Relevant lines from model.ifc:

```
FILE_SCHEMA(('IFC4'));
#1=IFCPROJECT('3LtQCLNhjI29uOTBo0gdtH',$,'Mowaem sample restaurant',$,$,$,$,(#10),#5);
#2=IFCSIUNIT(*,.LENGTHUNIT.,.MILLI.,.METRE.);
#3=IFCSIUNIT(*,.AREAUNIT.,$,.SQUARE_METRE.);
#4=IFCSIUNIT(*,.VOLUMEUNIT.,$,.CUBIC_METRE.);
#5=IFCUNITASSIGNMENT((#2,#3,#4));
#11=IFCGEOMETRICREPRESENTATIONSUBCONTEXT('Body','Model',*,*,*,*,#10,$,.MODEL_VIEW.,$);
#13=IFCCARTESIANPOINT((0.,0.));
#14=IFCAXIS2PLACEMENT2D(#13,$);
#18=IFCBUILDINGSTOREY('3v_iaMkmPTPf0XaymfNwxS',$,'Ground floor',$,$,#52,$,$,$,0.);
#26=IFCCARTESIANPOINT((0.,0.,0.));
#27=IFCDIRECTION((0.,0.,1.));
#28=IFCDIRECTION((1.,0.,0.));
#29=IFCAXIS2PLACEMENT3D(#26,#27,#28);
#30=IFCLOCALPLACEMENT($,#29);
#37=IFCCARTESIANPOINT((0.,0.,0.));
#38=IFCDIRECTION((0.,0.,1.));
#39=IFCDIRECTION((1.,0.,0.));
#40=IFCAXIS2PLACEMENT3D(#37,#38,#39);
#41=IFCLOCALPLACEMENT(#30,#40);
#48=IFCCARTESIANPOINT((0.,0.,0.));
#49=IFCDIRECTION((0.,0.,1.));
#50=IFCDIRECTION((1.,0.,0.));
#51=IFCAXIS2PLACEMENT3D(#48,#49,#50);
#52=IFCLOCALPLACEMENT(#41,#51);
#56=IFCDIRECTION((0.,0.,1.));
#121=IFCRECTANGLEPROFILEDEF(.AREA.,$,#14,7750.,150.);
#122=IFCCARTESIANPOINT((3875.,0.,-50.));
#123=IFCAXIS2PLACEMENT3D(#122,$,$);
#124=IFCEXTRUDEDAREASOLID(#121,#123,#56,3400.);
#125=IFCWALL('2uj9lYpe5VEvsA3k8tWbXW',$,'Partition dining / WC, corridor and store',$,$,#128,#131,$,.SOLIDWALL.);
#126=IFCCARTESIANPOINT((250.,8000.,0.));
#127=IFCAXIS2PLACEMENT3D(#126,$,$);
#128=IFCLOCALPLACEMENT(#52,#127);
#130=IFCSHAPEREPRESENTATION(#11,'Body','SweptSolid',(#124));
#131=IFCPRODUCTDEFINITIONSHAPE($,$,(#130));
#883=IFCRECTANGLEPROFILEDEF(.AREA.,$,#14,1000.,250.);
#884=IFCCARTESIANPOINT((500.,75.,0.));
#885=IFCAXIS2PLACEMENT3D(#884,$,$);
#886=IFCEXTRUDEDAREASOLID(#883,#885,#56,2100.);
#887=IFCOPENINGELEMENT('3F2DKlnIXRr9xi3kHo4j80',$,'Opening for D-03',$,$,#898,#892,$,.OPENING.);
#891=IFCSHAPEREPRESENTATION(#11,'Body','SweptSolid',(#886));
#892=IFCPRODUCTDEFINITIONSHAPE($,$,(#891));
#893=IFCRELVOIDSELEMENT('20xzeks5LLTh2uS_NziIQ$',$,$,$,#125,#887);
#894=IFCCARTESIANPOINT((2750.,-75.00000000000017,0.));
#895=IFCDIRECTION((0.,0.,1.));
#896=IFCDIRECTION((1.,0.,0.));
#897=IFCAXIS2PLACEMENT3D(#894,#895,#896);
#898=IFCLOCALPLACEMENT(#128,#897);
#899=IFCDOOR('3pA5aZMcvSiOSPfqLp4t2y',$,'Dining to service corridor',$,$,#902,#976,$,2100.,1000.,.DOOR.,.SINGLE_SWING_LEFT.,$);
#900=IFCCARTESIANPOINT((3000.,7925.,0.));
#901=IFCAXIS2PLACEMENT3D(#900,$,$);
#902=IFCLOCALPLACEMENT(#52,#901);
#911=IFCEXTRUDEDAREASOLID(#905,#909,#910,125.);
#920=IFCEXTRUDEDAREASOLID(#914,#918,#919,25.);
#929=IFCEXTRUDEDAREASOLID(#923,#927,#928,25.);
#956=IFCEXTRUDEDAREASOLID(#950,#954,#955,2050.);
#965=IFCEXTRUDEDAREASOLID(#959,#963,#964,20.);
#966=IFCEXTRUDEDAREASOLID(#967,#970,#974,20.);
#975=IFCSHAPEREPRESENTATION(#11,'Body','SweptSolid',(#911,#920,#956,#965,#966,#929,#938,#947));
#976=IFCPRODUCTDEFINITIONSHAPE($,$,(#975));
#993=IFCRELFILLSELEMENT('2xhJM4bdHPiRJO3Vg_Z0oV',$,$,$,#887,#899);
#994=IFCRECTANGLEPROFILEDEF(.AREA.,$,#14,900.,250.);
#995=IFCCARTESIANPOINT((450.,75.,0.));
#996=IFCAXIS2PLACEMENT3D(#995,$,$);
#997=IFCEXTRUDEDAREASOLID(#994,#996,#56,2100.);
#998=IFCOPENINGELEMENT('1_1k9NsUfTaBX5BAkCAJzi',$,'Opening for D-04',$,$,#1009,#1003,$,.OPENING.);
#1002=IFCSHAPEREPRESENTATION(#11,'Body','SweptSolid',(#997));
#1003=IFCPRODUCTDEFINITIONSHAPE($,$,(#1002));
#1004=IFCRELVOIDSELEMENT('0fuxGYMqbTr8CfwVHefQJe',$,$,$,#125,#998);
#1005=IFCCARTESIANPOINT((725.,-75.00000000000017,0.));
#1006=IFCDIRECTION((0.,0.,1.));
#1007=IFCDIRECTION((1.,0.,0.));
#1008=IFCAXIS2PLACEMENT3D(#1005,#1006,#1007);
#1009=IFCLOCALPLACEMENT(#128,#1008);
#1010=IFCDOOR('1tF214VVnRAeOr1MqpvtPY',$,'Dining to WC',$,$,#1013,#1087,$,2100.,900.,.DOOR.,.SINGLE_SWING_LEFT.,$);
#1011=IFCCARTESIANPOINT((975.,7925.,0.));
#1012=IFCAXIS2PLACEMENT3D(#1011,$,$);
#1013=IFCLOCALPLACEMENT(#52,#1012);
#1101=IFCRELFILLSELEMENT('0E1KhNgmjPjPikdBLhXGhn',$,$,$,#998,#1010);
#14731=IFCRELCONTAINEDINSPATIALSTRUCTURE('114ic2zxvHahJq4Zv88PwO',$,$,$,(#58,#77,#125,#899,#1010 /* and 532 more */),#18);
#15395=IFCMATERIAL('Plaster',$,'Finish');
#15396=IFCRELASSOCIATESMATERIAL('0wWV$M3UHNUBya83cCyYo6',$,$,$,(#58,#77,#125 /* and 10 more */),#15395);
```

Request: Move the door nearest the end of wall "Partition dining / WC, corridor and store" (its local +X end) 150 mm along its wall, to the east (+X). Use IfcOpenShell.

```python
import ifcopenshell
import ifcopenshell.api.geometry
import ifcopenshell.util.placement
import ifcopenshell.util.unit

model = ifcopenshell.open("model.ifc")
unit_scale = ifcopenshell.util.unit.calculate_unit_scale(model)

door = model.by_id(899)
opening = door.FillsVoids[0].RelatingOpeningElement
wall = opening.VoidsElements[0].RelatingBuildingElement

wall_matrix = ifcopenshell.util.placement.get_local_placement(wall.ObjectPlacement)
shift = wall_matrix[:3, 0] * 0.15 / unit_scale
before = ifcopenshell.util.placement.get_local_placement(door.ObjectPlacement)[:3, 3].copy()

# The door is not placed relative to its opening, so move both.
for product in (opening, door):
    matrix = ifcopenshell.util.placement.get_local_placement(product.ObjectPlacement)
    matrix[:3, 3] += shift
    ifcopenshell.api.geometry.edit_object_placement(model, product=product, matrix=matrix, is_si=False)

after = ifcopenshell.util.placement.get_local_placement(door.ObjectPlacement)[:3, 3]
print("door moved by", (after - before).round(3) + 0.0)

model.write("model_edited.ifc")
```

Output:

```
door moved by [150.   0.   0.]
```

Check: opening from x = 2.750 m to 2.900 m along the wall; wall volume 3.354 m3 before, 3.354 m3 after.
